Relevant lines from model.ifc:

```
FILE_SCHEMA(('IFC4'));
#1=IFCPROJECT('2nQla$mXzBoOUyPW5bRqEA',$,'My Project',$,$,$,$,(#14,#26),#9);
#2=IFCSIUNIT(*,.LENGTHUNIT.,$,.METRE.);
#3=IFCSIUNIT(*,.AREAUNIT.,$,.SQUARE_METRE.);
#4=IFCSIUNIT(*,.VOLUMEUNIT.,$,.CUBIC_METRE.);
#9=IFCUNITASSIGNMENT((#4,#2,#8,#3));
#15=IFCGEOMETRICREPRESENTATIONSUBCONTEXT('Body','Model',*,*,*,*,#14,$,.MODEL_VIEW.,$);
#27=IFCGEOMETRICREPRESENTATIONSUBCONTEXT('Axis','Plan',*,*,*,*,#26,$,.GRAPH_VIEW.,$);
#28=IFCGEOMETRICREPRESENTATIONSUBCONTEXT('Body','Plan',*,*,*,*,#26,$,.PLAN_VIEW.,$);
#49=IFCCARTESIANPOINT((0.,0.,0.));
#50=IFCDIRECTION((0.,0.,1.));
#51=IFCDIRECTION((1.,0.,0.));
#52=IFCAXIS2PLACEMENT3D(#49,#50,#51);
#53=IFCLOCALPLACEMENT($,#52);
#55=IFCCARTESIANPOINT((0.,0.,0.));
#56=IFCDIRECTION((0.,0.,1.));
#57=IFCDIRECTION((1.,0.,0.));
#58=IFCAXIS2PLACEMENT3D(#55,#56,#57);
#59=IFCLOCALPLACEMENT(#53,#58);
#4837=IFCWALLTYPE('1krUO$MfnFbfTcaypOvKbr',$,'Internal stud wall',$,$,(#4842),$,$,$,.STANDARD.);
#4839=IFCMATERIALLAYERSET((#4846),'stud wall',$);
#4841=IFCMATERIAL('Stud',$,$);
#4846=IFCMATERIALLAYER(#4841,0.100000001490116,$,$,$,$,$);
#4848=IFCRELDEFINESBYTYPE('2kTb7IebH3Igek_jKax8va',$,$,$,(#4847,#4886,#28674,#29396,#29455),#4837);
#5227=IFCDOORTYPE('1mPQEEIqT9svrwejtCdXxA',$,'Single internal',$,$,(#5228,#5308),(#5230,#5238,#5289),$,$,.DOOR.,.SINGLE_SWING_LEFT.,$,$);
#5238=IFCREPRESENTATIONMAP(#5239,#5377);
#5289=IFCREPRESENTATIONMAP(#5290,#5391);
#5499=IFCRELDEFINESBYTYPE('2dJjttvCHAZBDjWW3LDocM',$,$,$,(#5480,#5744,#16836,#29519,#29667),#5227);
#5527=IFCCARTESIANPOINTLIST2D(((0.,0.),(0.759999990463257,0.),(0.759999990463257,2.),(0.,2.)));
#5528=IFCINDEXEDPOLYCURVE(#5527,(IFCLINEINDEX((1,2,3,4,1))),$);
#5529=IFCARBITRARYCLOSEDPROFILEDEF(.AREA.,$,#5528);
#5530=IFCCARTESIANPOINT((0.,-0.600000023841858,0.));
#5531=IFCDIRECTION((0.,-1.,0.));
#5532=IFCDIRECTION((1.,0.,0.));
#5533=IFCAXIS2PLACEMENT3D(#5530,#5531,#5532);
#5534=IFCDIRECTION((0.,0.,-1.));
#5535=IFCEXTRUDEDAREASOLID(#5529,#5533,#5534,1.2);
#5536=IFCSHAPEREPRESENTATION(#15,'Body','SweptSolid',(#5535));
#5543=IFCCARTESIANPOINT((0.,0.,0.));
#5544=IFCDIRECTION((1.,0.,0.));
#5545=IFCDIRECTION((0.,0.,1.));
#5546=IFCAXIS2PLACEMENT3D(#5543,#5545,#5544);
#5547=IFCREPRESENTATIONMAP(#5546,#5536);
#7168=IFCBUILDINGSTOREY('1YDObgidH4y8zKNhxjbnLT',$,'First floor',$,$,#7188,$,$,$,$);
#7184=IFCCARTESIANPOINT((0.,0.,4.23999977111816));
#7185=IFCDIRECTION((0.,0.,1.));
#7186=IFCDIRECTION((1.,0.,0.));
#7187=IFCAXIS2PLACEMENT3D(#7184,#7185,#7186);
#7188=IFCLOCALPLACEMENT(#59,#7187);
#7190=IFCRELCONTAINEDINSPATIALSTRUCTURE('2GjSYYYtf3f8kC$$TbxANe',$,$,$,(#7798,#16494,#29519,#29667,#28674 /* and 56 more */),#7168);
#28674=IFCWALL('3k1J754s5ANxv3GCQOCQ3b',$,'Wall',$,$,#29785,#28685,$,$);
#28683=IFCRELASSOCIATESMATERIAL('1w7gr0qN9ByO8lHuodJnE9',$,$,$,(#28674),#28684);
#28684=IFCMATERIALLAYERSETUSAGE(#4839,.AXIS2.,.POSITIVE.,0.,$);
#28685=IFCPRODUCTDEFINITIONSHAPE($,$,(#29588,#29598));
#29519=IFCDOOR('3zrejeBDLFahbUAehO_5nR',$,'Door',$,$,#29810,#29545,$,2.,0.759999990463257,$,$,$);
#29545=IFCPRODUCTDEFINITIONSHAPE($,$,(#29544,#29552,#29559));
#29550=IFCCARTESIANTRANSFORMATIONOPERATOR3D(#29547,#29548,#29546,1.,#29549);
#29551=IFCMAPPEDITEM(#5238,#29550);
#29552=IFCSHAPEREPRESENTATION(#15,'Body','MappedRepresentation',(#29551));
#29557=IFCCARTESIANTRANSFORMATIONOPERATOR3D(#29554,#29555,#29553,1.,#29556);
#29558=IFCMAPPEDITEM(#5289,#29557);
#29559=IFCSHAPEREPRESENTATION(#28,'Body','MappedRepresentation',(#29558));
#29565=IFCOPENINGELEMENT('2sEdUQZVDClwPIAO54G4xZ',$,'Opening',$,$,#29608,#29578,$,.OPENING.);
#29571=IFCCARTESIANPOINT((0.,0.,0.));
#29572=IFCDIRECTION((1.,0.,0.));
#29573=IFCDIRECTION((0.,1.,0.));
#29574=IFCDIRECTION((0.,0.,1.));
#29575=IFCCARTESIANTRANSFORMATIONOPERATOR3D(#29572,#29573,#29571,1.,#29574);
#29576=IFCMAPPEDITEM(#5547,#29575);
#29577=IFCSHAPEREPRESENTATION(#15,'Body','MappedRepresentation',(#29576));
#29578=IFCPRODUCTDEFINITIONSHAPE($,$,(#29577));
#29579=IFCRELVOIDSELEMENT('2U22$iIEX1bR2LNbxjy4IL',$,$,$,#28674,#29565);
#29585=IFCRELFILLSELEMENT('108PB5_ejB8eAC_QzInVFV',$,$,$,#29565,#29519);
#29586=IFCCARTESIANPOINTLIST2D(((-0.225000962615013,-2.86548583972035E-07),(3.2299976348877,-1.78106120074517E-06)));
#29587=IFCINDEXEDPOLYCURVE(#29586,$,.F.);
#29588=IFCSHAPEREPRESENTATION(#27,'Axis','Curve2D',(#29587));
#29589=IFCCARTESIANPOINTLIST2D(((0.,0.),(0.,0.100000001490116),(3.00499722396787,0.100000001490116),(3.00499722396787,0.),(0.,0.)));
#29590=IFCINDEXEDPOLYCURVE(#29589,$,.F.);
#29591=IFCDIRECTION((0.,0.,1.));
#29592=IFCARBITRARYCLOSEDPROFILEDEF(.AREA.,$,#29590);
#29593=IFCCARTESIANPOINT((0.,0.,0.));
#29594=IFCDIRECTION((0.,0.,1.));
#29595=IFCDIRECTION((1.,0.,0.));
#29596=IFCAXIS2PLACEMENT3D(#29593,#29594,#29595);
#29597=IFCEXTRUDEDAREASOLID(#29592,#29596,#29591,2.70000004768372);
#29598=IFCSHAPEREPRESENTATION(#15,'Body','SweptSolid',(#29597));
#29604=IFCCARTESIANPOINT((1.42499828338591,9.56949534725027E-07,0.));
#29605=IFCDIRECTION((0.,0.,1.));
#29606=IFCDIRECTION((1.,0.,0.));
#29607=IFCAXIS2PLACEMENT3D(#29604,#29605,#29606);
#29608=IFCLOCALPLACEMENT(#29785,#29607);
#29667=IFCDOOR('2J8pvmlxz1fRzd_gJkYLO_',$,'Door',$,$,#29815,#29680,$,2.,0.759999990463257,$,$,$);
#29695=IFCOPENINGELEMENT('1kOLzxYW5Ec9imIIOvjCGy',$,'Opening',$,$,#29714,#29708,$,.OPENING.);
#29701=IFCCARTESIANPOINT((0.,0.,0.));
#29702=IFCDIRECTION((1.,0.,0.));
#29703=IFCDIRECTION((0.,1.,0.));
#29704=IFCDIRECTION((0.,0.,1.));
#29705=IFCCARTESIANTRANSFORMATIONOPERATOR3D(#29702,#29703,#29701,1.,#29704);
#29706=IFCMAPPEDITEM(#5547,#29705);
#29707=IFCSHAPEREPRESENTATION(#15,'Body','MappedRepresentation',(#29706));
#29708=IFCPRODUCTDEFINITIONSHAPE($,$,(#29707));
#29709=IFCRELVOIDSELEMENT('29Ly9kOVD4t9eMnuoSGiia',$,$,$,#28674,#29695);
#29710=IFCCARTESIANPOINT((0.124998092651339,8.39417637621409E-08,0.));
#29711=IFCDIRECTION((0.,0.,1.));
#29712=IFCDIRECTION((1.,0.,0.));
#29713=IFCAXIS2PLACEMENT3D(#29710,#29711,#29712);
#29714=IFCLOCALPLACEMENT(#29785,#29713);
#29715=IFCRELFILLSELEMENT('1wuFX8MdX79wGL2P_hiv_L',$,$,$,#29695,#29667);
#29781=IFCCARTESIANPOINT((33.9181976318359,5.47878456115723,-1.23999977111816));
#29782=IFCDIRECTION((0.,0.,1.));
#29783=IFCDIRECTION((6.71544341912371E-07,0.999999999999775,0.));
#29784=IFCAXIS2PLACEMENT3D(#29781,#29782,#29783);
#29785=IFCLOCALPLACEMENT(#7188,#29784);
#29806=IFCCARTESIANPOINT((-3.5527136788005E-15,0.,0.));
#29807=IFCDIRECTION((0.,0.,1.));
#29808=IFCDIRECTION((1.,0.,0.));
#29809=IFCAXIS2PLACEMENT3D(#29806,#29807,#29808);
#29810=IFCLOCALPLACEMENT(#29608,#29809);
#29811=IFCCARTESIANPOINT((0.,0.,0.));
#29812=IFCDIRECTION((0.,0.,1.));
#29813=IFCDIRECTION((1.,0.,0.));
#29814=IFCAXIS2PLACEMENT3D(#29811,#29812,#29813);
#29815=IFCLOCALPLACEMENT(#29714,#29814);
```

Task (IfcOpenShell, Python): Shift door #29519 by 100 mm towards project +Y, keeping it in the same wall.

```python
import ifcopenshell
import ifcopenshell.api.geometry
import ifcopenshell.util.placement
import ifcopenshell.util.unit

model = ifcopenshell.open("model.ifc")
unit_scale = ifcopenshell.util.unit.calculate_unit_scale(model)

door = model.by_guid("3zrejeBDLFahbUAehO_5nR")
opening = door.FillsVoids[0].RelatingOpeningElement
wall = opening.VoidsElements[0].RelatingBuildingElement

wall_matrix = ifcopenshell.util.placement.get_local_placement(wall.ObjectPlacement)
shift = wall_matrix[:3, 0] * 0.1 / unit_scale
before = ifcopenshell.util.placement.get_local_placement(door.ObjectPlacement)[:3, 3].copy()

# The door is placed relative to its opening, so it follows when the opening moves.
matrix = ifcopenshell.util.placement.get_local_placement(opening.ObjectPlacement)
matrix[:3, 3] += shift
ifcopenshell.api.geometry.edit_object_placement(
    model, product=opening, matrix=matrix, is_si=False, should_transform_children=True
)

after = ifcopenshell.util.placement.get_local_placement(door.ObjectPlacement)[:3, 3]
print("door moved by", (after - before).round(3) + 0.0)

model.write("model_edited.ifc")
```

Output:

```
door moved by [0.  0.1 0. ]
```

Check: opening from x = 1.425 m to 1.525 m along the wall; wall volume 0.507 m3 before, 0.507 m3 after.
